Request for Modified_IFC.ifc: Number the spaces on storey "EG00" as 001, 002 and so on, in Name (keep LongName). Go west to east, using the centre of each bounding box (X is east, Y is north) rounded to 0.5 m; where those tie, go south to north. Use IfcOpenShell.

First a look at what the model holds.

```python
import ifcopenshell
import ifcopenshell.util.element
import ifcopenshell.util.placement

model = ifcopenshell.open("Modified_IFC.ifc")
print(model.schema)
storey = next(s for s in model.by_type("IfcBuildingStorey") if s.Name == "EG00")
spaces = [e for e in ifcopenshell.util.element.get_decomposition(storey) if e.is_a("IfcSpace")]
for e in sorted(spaces, key=lambda e: e.id()):
    origin = ifcopenshell.util.placement.get_local_placement(e.ObjectPlacement)[:3, 3]
    print(e.id(), e.Name, e.LongName, origin.round(2) + 0.0, sep=" | ")
```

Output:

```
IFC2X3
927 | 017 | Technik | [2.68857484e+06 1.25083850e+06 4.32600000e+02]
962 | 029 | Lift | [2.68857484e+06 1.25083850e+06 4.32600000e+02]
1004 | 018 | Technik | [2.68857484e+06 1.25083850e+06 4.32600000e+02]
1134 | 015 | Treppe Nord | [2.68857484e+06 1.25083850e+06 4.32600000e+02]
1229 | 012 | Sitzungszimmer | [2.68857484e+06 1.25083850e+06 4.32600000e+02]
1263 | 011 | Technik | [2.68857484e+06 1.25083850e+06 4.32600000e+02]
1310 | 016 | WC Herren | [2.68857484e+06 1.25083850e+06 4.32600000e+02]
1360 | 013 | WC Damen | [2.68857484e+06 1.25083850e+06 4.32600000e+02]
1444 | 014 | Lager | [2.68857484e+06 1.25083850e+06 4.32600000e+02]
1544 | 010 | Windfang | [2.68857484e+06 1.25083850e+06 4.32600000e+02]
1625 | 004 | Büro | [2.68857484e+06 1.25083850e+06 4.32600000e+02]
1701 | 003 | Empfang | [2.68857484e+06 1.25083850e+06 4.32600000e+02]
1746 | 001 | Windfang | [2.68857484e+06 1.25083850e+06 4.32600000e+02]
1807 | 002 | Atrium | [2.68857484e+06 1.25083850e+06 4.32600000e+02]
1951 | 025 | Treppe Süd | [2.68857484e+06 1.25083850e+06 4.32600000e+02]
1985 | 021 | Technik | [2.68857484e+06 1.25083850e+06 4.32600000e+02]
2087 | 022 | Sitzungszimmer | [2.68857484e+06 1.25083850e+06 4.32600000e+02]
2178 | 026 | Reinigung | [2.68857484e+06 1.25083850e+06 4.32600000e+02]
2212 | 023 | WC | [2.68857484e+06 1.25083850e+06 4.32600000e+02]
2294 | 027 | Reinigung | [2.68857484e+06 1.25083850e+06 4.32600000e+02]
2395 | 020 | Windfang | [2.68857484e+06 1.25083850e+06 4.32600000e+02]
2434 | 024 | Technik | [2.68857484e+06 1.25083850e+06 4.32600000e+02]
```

```python
import ifcopenshell
import ifcopenshell.geom
import ifcopenshell.util.element
import ifcopenshell.util.shape

model = ifcopenshell.open("Modified_IFC.ifc")
settings = ifcopenshell.geom.settings()
settings.set("use-world-coords", True)


def centre(element):
    shape = ifcopenshell.geom.create_shape(settings, element)
    return ifcopenshell.util.shape.get_bbox_centroid(shape.geometry)


storey = next(s for s in model.by_type("IfcBuildingStorey") if s.Name == "EG00")
spaces = [e for e in ifcopenshell.util.element.get_decomposition(storey) if e.is_a("IfcSpace")]

# Insertion points can sit at a corner or the storey origin, so sort by the geometry (in metres).
centres = {e: centre(e) for e in spaces}
spaces.sort(key=lambda e: (round(centres[e][0] / 0.5), centres[e][1]))

for i, e in enumerate(spaces, start=1):
    number = f"0{i:02d}"
    e.Name = number
    print(e.id(), number)

model.write("Modified_IFC_v2.ifc")
```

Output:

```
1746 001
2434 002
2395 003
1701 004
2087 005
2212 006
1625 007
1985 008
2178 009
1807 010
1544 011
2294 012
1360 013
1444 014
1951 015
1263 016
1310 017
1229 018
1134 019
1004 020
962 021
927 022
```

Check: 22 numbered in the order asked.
